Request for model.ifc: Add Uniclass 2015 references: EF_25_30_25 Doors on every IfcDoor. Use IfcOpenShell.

First a look at what the model holds.

```python
import ifcopenshell

model = ifcopenshell.open("model.ifc")
print(model.schema)
print("classifications:", [c.Name for c in model.by_type("IfcClassification")])
for ifc_class in ("IfcDoor", "IfcRoof", "IfcStair", "IfcWall", "IfcWindow"):
    print(ifc_class, len(model.by_type(ifc_class)))
```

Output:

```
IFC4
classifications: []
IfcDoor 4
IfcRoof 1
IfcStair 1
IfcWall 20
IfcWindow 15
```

```python
import ifcopenshell
import ifcopenshell.api.classification

model = ifcopenshell.open("model.ifc")

system = ifcopenshell.api.classification.add_classification(model, classification="Uniclass 2015")

codes = {
    "IfcDoor": ("EF_25_30_25", "Doors"),
}
for ifc_class, (code, name) in codes.items():
    products = model.by_type(ifc_class)
    ifcopenshell.api.classification.add_reference(
        model, products=products, classification=system, identification=code, name=name
    )
    print(code, len(products))

model.write("model_rev.ifc")
```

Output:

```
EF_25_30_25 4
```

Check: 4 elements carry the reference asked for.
